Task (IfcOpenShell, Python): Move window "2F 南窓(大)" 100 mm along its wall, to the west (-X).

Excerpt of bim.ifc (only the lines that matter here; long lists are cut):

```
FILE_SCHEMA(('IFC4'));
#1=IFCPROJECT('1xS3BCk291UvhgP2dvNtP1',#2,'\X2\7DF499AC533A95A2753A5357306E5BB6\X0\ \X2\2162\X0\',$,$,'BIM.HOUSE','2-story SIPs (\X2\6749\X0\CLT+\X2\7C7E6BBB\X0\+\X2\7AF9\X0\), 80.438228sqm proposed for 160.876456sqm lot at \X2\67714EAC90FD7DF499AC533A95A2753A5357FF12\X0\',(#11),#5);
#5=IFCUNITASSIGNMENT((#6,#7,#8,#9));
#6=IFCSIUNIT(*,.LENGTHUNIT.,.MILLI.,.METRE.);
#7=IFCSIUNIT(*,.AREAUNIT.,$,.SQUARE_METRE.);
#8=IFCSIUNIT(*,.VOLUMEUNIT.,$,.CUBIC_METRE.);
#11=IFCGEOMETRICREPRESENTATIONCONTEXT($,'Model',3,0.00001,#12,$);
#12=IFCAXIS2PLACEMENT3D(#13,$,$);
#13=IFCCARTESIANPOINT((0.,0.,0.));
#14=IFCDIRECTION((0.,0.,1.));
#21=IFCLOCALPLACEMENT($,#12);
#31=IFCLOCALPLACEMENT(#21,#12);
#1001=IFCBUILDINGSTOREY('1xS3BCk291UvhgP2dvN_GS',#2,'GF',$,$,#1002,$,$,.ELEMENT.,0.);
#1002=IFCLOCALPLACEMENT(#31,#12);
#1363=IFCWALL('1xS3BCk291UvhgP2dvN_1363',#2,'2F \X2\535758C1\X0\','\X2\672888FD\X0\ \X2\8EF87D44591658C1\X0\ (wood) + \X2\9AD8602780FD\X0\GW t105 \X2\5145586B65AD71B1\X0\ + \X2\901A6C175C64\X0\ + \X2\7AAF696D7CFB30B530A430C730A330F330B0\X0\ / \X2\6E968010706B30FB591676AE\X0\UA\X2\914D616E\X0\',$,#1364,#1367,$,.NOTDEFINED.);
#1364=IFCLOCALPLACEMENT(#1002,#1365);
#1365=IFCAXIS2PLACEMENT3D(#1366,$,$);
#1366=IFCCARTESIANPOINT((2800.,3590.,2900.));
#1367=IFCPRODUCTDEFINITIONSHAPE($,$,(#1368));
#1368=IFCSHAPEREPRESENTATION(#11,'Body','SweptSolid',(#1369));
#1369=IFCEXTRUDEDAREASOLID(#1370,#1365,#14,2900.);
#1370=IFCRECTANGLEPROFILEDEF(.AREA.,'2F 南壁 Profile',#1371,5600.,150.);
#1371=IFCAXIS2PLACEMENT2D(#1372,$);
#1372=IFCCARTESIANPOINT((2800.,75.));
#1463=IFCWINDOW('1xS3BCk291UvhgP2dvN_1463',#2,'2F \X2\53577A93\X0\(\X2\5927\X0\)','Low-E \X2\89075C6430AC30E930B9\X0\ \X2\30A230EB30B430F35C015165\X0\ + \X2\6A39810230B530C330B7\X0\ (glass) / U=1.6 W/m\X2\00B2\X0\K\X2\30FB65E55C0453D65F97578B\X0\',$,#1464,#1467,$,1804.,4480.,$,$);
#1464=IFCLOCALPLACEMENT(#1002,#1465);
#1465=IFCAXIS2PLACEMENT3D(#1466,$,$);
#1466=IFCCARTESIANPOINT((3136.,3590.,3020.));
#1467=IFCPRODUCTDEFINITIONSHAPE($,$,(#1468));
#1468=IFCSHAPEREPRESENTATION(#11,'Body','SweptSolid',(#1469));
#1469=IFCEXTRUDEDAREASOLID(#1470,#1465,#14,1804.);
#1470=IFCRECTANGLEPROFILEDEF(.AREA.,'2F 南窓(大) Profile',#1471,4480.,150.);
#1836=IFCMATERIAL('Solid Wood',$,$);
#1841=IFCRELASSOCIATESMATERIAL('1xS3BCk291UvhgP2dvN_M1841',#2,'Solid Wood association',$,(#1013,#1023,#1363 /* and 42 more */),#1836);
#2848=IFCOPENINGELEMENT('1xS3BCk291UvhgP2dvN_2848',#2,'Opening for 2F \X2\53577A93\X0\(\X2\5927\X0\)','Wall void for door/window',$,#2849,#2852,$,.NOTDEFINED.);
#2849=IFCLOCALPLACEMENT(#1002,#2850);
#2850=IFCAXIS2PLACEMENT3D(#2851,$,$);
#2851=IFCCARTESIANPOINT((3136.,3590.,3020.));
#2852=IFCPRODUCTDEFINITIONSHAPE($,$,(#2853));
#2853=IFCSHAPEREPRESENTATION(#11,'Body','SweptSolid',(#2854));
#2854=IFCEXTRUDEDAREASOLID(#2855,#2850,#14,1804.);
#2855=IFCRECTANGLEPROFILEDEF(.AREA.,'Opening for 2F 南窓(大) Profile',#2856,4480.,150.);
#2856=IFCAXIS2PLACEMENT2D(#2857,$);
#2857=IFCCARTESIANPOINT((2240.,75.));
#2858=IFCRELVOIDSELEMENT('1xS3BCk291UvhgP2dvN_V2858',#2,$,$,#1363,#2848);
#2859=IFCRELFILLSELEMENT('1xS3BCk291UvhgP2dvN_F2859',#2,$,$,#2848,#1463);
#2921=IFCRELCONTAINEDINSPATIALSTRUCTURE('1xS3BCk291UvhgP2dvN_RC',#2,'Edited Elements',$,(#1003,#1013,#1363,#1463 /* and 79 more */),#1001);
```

```python
import ifcopenshell
import ifcopenshell.api.geometry
import ifcopenshell.util.placement

model = ifcopenshell.open("bim.ifc")

window = model.by_id(1463)
opening = window.FillsVoids[0].RelatingOpeningElement
wall = opening.VoidsElements[0].RelatingBuildingElement

wall_matrix = ifcopenshell.util.placement.get_local_placement(wall.ObjectPlacement)
shift = wall_matrix[:3, 0] * -100.0
before = ifcopenshell.util.placement.get_local_placement(window.ObjectPlacement)[:3, 3].copy()

# The window is not placed relative to its opening, so move both.
for product in (opening, window):
    matrix = ifcopenshell.util.placement.get_local_placement(product.ObjectPlacement)
    matrix[:3, 3] += shift
    ifcopenshell.api.geometry.edit_object_placement(model, product=product, matrix=matrix, is_si=False)

after = ifcopenshell.util.placement.get_local_placement(window.ObjectPlacement)[:3, 3]
print("window moved by", (after - before).round(3) + 0.0)

model.write("bim_v2.ifc")
```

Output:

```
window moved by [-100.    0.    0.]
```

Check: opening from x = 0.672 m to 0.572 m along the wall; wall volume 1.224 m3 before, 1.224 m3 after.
